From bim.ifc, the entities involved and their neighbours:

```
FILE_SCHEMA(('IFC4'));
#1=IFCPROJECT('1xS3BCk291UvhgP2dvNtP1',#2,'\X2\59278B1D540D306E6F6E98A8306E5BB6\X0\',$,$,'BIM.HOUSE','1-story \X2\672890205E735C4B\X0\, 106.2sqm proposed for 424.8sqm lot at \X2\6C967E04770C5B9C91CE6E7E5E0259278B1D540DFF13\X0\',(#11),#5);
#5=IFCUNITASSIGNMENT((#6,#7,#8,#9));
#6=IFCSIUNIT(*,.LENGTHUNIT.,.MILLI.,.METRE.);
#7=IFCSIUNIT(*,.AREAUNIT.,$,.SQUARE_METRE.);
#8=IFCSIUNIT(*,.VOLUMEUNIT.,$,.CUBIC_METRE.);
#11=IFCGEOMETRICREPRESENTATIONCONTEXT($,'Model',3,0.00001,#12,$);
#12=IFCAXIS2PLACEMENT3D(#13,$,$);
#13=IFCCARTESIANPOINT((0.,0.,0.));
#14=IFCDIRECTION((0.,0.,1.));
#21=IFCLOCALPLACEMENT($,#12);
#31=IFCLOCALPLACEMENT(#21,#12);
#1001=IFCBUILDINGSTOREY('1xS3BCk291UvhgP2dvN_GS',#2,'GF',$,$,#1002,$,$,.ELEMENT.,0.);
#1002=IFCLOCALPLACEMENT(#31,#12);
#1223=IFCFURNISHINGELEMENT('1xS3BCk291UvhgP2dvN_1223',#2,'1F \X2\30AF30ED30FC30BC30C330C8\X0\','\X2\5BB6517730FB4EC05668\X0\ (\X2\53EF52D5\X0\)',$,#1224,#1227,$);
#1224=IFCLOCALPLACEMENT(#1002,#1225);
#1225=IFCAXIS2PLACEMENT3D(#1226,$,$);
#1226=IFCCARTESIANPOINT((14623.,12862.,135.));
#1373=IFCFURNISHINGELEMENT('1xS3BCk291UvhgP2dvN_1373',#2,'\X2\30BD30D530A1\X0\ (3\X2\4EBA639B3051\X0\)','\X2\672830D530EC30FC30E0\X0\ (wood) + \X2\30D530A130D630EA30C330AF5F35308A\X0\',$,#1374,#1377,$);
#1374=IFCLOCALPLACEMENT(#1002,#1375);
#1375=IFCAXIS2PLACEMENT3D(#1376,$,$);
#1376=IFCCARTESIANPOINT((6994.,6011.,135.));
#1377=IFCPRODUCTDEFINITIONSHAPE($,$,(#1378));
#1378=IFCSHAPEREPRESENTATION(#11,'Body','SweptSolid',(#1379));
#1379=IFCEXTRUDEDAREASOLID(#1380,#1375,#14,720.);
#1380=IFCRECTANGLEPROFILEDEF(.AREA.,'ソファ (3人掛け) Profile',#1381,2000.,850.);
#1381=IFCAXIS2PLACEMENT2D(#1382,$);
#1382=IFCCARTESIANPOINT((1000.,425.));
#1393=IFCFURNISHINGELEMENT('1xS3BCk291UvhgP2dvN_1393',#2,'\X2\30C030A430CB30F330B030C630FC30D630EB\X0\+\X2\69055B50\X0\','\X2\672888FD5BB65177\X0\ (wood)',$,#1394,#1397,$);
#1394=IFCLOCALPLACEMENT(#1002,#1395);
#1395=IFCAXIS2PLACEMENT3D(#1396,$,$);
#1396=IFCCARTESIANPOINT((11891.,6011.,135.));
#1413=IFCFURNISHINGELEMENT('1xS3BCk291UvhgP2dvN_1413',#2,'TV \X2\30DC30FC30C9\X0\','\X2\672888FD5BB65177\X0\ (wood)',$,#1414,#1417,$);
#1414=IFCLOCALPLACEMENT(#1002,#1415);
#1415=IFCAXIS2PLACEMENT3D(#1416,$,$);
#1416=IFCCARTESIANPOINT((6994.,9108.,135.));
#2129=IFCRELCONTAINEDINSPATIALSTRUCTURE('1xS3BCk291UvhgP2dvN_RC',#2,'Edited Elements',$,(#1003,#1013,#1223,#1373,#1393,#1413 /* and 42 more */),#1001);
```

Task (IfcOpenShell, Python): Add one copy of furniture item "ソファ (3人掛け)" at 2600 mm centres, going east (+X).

```python
import numpy as np
import ifcopenshell
import ifcopenshell.api.geometry
import ifcopenshell.api.root
import ifcopenshell.util.element
import ifcopenshell.util.placement

model = ifcopenshell.open("bim.ifc")


def reuse_history(source, copy):
    """copy_class also copies each property set's owner history, people and application; keep the originals."""
    for rel in copy.IsDefinedBy:
        if rel.is_a("IfcRelDefinesByProperties") and (history := rel.RelatingPropertyDefinition.OwnerHistory):
            rel.RelatingPropertyDefinition.OwnerHistory = source.OwnerHistory
            ifcopenshell.util.element.remove_deep2(model, history)


source = model.by_guid("1xS3BCk291UvhgP2dvN_1373")
base = ifcopenshell.util.placement.get_local_placement(source.ObjectPlacement)
step = np.array([1.0, 0.0, 0.0]) * 2600.0

for i in range(1, 2):
    copy = ifcopenshell.api.root.copy_class(model, product=source)
    copy.Representation = ifcopenshell.util.element.copy_deep(
        model, source.Representation, exclude=["IfcGeometricRepresentationContext", "IfcRepresentationMap"]
    )
    reuse_history(source, copy)
    matrix = base.copy()
    matrix[:3, 3] += i * step
    print("added at", matrix[:3, 3].round(3) + 0.0)
    ifcopenshell.api.geometry.edit_object_placement(model, product=copy, matrix=matrix, is_si=False)

model.write("bim_edited.ifc")
```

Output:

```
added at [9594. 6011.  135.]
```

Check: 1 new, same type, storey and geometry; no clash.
